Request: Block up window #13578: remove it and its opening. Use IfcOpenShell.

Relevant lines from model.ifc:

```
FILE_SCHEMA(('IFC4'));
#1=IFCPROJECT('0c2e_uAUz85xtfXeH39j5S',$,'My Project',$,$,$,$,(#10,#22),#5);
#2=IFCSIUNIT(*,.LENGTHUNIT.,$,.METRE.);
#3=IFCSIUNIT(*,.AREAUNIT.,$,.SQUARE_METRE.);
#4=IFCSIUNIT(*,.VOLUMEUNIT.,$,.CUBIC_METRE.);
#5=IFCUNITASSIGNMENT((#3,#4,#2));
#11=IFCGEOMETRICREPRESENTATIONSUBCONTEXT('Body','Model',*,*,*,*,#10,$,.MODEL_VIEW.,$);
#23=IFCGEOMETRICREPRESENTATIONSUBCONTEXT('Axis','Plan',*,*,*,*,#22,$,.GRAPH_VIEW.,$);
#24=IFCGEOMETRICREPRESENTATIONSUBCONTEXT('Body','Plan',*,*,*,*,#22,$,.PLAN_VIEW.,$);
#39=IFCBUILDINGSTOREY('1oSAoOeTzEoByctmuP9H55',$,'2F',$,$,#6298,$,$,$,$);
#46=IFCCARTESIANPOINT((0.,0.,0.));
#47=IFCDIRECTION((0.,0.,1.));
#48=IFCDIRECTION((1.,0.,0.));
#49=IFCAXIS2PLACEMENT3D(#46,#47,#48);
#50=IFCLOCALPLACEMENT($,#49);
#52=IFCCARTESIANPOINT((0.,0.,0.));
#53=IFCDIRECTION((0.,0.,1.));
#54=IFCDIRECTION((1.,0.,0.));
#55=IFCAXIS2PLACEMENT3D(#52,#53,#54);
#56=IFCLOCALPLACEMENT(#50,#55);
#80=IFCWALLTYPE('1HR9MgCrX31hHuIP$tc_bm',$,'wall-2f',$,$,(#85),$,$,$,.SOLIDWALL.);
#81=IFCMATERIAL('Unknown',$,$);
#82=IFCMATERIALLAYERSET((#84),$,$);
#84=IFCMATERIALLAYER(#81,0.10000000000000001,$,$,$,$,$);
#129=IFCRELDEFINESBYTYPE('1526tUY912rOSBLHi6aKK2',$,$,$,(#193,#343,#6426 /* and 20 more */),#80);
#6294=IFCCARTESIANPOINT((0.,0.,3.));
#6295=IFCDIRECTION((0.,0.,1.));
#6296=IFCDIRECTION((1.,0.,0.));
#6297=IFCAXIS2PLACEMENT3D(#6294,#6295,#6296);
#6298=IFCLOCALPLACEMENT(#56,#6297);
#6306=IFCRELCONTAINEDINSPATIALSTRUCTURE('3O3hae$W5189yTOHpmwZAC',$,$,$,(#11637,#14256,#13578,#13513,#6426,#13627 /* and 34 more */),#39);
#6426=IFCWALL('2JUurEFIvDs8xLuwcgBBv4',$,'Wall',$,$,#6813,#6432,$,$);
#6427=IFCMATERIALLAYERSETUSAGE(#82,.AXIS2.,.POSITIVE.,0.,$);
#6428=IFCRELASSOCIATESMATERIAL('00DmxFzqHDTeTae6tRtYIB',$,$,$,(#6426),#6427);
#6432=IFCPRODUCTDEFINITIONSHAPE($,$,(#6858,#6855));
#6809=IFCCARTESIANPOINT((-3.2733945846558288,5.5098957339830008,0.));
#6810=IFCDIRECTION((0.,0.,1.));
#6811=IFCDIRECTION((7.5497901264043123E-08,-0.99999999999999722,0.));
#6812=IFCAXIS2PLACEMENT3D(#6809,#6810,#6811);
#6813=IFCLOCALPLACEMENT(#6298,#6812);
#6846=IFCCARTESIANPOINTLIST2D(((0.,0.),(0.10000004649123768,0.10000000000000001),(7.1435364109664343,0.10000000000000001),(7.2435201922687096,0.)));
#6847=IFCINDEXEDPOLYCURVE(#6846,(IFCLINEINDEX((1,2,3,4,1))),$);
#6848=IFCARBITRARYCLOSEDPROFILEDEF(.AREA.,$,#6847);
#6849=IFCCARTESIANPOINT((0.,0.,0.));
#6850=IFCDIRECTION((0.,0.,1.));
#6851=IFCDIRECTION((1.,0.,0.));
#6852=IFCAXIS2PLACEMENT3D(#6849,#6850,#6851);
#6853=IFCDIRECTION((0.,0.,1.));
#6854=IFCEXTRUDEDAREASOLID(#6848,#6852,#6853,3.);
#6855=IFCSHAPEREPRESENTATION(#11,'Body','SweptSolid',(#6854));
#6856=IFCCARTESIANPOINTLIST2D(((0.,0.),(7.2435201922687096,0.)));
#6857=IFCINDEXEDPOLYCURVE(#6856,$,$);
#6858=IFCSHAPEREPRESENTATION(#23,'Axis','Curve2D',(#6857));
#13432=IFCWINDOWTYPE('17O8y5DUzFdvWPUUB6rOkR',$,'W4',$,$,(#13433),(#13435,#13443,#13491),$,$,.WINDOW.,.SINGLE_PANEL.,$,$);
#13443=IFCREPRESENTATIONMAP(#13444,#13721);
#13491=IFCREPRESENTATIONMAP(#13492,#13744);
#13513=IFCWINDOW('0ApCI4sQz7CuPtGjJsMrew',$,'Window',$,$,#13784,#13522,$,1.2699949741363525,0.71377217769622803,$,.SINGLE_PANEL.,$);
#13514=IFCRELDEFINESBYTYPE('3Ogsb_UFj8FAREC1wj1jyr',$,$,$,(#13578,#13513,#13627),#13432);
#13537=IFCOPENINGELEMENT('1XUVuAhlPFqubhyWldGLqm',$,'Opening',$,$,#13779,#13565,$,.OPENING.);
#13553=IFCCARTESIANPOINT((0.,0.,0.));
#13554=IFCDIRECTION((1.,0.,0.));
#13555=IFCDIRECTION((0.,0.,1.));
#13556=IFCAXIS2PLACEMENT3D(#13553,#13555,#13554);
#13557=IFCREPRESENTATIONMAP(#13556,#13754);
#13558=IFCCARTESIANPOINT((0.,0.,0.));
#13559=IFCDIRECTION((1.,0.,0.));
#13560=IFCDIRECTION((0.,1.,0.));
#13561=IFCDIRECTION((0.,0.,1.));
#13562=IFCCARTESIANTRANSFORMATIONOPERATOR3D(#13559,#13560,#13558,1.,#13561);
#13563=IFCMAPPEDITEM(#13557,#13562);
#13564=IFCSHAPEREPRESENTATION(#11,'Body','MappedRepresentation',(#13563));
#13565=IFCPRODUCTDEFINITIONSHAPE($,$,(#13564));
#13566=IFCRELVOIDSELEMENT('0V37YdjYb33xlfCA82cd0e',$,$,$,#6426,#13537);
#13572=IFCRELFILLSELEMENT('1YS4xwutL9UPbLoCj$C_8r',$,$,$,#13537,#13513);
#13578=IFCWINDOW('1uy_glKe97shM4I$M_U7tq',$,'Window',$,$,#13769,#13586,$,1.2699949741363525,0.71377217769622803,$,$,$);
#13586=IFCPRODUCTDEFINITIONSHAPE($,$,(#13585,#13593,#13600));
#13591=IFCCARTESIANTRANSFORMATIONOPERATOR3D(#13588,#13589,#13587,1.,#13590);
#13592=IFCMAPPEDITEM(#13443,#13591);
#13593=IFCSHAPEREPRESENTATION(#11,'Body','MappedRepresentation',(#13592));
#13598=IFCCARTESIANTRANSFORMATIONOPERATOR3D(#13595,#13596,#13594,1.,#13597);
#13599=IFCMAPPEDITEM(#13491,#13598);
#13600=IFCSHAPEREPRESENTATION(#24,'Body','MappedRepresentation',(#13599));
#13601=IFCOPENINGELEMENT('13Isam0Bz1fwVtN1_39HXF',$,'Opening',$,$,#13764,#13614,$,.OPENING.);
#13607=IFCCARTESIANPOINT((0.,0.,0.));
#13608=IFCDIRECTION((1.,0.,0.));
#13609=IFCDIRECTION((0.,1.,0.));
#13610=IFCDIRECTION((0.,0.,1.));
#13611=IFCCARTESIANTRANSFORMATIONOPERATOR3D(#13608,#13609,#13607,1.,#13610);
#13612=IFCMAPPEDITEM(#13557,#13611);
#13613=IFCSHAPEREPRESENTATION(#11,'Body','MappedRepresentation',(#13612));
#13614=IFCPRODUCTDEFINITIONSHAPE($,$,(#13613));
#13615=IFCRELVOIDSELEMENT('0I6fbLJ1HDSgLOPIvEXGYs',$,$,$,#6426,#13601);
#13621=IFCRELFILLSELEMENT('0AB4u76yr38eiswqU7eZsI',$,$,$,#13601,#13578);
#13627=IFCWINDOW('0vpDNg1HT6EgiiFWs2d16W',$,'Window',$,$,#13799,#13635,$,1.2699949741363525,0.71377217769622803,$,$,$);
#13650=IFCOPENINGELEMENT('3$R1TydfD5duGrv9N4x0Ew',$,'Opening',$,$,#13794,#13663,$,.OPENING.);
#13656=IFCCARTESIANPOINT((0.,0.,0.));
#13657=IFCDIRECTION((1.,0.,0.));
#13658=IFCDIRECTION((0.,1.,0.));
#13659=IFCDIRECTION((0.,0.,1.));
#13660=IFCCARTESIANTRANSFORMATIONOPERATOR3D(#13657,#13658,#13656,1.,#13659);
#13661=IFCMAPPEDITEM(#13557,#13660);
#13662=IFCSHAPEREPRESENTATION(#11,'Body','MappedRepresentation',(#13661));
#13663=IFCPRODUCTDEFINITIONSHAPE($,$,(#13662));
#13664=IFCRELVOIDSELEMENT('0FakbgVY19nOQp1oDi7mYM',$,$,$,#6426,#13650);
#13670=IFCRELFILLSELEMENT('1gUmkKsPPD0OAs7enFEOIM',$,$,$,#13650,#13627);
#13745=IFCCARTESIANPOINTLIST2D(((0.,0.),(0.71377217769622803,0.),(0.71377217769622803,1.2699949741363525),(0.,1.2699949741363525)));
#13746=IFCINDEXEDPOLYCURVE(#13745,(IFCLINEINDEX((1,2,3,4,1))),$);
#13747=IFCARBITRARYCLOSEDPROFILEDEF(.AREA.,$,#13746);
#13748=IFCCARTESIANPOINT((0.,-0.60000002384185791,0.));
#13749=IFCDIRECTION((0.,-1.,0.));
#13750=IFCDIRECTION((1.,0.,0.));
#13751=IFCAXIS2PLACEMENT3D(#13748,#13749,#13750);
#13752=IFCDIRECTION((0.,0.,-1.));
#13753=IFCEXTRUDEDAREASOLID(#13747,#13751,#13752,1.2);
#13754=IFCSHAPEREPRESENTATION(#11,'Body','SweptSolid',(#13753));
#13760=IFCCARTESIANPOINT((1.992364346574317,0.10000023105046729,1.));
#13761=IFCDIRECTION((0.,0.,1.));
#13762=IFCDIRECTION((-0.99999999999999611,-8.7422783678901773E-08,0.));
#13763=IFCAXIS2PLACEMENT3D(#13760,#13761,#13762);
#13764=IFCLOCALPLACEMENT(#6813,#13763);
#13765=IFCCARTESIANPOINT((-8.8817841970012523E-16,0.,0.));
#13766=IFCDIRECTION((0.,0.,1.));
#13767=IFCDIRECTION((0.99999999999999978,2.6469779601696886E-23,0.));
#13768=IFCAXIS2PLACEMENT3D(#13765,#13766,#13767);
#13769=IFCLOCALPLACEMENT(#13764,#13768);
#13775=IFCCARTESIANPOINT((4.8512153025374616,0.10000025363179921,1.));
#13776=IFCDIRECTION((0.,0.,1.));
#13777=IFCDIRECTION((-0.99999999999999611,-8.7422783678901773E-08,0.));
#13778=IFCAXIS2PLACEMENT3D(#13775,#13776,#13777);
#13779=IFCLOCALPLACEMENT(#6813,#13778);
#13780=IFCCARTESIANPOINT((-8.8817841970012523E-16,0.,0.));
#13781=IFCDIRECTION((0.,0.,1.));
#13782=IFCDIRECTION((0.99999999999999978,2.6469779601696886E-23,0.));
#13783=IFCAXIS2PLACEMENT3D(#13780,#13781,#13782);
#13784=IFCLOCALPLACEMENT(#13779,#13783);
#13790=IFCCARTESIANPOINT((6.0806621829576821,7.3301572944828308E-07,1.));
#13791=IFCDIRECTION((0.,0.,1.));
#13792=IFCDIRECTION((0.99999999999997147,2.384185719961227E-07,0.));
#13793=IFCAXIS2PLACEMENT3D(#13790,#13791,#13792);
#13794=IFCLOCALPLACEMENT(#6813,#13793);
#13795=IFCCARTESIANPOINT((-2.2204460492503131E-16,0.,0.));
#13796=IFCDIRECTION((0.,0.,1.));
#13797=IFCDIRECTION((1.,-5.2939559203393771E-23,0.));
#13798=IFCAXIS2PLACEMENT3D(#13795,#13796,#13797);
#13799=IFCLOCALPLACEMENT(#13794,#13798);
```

```python
import ifcopenshell
import ifcopenshell.api.feature
import ifcopenshell.api.root
import ifcopenshell.geom
import ifcopenshell.util.shape

model = ifcopenshell.open("model.ifc")
settings = ifcopenshell.geom.settings()


def volume(element):
    """Net volume in cubic metres, openings subtracted."""
    shape = ifcopenshell.geom.create_shape(settings, element)
    return ifcopenshell.util.shape.get_volume(shape.geometry)


window = model.by_id(13578)
opening = window.FillsVoids[0].RelatingOpeningElement
wall = opening.VoidsElements[0].RelatingBuildingElement
before = volume(wall)

ifcopenshell.api.root.remove_product(model, product=window)
ifcopenshell.api.feature.remove_feature(model, feature=opening)

after = volume(wall)

print(f"wall volume {before:.3f} -> {after:.3f} m3")

model.write("model_edited.ifc")
```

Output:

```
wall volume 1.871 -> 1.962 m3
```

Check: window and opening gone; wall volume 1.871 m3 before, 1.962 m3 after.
